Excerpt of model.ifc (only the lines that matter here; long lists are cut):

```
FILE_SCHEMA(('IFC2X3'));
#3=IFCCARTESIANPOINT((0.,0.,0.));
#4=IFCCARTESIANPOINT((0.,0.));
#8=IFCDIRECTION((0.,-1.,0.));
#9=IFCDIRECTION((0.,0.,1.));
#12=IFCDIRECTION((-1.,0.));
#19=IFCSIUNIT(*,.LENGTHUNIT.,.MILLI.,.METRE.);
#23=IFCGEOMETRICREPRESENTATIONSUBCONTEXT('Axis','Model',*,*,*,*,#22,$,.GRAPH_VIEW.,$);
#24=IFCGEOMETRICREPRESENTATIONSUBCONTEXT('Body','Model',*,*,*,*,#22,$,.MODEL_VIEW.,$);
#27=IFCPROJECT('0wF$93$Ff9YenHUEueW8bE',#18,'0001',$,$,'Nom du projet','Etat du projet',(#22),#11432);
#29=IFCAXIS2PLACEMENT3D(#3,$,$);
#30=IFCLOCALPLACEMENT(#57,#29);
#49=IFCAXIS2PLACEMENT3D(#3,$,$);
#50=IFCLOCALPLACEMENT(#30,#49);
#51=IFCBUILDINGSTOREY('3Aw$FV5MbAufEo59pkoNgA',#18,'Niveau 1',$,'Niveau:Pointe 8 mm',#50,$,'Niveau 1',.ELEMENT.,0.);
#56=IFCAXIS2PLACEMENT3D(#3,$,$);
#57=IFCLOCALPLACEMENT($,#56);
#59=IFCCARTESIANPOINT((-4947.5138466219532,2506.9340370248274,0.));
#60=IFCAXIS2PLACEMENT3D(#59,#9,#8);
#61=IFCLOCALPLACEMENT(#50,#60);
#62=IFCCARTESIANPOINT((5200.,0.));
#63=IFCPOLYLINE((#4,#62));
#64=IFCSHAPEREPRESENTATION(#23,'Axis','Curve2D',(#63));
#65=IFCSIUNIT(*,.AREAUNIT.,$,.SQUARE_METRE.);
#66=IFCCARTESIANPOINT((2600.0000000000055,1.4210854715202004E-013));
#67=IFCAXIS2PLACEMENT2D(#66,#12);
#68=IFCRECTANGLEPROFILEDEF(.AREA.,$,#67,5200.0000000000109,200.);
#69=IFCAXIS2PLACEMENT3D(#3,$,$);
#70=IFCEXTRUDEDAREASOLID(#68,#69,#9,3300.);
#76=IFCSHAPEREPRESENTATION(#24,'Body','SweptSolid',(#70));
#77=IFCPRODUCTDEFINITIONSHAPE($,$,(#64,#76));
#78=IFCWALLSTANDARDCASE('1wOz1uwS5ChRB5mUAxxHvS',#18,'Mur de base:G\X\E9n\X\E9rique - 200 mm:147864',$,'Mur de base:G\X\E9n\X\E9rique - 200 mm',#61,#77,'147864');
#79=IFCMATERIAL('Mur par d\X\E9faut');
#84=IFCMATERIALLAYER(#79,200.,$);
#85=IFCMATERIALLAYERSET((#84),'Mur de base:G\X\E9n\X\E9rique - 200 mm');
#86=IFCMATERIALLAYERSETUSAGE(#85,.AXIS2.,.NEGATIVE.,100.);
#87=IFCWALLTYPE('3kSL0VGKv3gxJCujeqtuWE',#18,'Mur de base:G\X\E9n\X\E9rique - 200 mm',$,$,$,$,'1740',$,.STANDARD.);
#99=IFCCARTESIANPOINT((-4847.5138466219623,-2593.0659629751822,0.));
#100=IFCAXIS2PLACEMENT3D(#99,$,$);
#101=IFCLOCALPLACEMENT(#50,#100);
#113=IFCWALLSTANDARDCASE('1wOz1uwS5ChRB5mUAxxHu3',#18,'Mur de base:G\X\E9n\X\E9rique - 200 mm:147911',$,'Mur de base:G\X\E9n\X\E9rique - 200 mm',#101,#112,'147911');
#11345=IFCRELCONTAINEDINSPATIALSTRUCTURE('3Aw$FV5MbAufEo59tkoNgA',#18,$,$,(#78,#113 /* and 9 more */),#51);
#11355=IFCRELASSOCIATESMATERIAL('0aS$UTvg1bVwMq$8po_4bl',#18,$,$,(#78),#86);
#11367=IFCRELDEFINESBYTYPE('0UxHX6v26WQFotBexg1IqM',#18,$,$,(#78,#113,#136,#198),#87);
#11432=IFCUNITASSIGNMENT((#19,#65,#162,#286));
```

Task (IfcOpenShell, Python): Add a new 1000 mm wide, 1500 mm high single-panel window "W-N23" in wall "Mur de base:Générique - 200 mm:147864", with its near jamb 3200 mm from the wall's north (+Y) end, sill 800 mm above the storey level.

```python
import numpy as np
import ifcopenshell
import ifcopenshell.api.feature
import ifcopenshell.api.geometry
import ifcopenshell.api.root
import ifcopenshell.api.spatial
import ifcopenshell.api.type
import ifcopenshell.geom
import ifcopenshell.util.element
import ifcopenshell.util.placement
import ifcopenshell.util.representation
import ifcopenshell.util.shape
import ifcopenshell.util.unit

model = ifcopenshell.open("model.ifc")
unit_scale = ifcopenshell.util.unit.calculate_unit_scale(model)
settings = ifcopenshell.geom.settings()


def volume(element):
    """Net volume in cubic metres, openings subtracted."""
    shape = ifcopenshell.geom.create_shape(settings, element)
    return ifcopenshell.util.shape.get_volume(shape.geometry)


wall = model.by_guid("1wOz1uwS5ChRB5mUAxxHvS")
storey = ifcopenshell.util.element.get_container(wall, ifc_class="IfcBuildingStorey")
context = ifcopenshell.util.representation.get_context(model, "Model", "Body", "MODEL_VIEW")
before = volume(wall)

width, height, from_end, sill = 1, 1.5, 3.2, 0.8  # metres

# The wall runs along its own X axis, and the end named is its -X end.
wall_shape = ifcopenshell.geom.create_shape(settings, wall)
x, y, z = ifcopenshell.util.shape.get_vertices(wall_shape.geometry).T
start = x.min() + from_end
face, thickness = float(y.min()), float(y.max() - y.min())
wall_matrix = ifcopenshell.util.placement.get_local_placement(wall.ObjectPlacement)
level = ifcopenshell.util.placement.get_local_placement(storey.ObjectPlacement)[2, 3]


def in_wall(x, y):
    """Placement at x, y metres in the wall's axes, at sill height."""
    matrix = wall_matrix.copy()
    matrix[:, 3] = wall_matrix @ np.array([x / unit_scale, y / unit_scale, 0.0, 1.0])
    matrix[2, 3] = level + sill / unit_scale
    return matrix


# Opening: a box that overshoots both wall faces by 50 mm.
opening = ifcopenshell.api.root.create_entity(model, ifc_class="IfcOpeningElement")
box = ifcopenshell.api.geometry.add_wall_representation(
    model, context=context, length=width, height=height, thickness=thickness + 0.1
)
ifcopenshell.api.geometry.assign_representation(model, product=opening, representation=box)
ifcopenshell.api.geometry.edit_object_placement(model, product=opening, matrix=in_wall(start, face - 0.05), is_si=False)
ifcopenshell.api.feature.add_feature(model, feature=opening, element=wall)

window = ifcopenshell.api.root.create_entity(model, ifc_class="IfcWindow", name="W-N23")
window.OverallWidth, window.OverallHeight = width / unit_scale, height / unit_scale
body = ifcopenshell.api.geometry.add_window_representation(
    model,
    context=context,
    overall_width=window.OverallWidth,
    overall_height=window.OverallHeight,
    partition_type="SINGLE_PANEL",
)
ifcopenshell.api.geometry.assign_representation(model, product=window, representation=body)
ifcopenshell.api.spatial.assign_container(model, products=[window], relating_structure=storey)
fills = ifcopenshell.api.feature.add_filling(model, opening=opening, element=window)
fills.OwnerHistory = window.OwnerHistory  # required in IFC2X3

# IFC2X3 keeps the operation on the window style.
style = ifcopenshell.api.root.create_entity(model, ifc_class="IfcWindowStyle", name="W-N23")
style.OperationType, style.ConstructionType = "SINGLE_PANEL", "NOTDEFINED"
style.ParameterTakesPrecedence = style.Sizeable = False
ifcopenshell.api.type.assign_type(model, related_objects=[window], relating_type=style)

# Centre the window in the wall's thickness.
ifcopenshell.api.geometry.edit_object_placement(model, product=window, matrix=in_wall(start, face), is_si=False)
window_shape = ifcopenshell.geom.create_shape(settings, window)
depth = ifcopenshell.util.shape.get_vertices(window_shape.geometry)[:, 1]
offset = face + thickness / 2 - (depth.min() + depth.max()) / 2
ifcopenshell.api.geometry.edit_object_placement(model, product=window, matrix=in_wall(start, offset), is_si=False)

after = volume(wall)

print(f"wall volume {before:.3f} -> {after:.3f} m3")

model.write("model_rev.ifc")
```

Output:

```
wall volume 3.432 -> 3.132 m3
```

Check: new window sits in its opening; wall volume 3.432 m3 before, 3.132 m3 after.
